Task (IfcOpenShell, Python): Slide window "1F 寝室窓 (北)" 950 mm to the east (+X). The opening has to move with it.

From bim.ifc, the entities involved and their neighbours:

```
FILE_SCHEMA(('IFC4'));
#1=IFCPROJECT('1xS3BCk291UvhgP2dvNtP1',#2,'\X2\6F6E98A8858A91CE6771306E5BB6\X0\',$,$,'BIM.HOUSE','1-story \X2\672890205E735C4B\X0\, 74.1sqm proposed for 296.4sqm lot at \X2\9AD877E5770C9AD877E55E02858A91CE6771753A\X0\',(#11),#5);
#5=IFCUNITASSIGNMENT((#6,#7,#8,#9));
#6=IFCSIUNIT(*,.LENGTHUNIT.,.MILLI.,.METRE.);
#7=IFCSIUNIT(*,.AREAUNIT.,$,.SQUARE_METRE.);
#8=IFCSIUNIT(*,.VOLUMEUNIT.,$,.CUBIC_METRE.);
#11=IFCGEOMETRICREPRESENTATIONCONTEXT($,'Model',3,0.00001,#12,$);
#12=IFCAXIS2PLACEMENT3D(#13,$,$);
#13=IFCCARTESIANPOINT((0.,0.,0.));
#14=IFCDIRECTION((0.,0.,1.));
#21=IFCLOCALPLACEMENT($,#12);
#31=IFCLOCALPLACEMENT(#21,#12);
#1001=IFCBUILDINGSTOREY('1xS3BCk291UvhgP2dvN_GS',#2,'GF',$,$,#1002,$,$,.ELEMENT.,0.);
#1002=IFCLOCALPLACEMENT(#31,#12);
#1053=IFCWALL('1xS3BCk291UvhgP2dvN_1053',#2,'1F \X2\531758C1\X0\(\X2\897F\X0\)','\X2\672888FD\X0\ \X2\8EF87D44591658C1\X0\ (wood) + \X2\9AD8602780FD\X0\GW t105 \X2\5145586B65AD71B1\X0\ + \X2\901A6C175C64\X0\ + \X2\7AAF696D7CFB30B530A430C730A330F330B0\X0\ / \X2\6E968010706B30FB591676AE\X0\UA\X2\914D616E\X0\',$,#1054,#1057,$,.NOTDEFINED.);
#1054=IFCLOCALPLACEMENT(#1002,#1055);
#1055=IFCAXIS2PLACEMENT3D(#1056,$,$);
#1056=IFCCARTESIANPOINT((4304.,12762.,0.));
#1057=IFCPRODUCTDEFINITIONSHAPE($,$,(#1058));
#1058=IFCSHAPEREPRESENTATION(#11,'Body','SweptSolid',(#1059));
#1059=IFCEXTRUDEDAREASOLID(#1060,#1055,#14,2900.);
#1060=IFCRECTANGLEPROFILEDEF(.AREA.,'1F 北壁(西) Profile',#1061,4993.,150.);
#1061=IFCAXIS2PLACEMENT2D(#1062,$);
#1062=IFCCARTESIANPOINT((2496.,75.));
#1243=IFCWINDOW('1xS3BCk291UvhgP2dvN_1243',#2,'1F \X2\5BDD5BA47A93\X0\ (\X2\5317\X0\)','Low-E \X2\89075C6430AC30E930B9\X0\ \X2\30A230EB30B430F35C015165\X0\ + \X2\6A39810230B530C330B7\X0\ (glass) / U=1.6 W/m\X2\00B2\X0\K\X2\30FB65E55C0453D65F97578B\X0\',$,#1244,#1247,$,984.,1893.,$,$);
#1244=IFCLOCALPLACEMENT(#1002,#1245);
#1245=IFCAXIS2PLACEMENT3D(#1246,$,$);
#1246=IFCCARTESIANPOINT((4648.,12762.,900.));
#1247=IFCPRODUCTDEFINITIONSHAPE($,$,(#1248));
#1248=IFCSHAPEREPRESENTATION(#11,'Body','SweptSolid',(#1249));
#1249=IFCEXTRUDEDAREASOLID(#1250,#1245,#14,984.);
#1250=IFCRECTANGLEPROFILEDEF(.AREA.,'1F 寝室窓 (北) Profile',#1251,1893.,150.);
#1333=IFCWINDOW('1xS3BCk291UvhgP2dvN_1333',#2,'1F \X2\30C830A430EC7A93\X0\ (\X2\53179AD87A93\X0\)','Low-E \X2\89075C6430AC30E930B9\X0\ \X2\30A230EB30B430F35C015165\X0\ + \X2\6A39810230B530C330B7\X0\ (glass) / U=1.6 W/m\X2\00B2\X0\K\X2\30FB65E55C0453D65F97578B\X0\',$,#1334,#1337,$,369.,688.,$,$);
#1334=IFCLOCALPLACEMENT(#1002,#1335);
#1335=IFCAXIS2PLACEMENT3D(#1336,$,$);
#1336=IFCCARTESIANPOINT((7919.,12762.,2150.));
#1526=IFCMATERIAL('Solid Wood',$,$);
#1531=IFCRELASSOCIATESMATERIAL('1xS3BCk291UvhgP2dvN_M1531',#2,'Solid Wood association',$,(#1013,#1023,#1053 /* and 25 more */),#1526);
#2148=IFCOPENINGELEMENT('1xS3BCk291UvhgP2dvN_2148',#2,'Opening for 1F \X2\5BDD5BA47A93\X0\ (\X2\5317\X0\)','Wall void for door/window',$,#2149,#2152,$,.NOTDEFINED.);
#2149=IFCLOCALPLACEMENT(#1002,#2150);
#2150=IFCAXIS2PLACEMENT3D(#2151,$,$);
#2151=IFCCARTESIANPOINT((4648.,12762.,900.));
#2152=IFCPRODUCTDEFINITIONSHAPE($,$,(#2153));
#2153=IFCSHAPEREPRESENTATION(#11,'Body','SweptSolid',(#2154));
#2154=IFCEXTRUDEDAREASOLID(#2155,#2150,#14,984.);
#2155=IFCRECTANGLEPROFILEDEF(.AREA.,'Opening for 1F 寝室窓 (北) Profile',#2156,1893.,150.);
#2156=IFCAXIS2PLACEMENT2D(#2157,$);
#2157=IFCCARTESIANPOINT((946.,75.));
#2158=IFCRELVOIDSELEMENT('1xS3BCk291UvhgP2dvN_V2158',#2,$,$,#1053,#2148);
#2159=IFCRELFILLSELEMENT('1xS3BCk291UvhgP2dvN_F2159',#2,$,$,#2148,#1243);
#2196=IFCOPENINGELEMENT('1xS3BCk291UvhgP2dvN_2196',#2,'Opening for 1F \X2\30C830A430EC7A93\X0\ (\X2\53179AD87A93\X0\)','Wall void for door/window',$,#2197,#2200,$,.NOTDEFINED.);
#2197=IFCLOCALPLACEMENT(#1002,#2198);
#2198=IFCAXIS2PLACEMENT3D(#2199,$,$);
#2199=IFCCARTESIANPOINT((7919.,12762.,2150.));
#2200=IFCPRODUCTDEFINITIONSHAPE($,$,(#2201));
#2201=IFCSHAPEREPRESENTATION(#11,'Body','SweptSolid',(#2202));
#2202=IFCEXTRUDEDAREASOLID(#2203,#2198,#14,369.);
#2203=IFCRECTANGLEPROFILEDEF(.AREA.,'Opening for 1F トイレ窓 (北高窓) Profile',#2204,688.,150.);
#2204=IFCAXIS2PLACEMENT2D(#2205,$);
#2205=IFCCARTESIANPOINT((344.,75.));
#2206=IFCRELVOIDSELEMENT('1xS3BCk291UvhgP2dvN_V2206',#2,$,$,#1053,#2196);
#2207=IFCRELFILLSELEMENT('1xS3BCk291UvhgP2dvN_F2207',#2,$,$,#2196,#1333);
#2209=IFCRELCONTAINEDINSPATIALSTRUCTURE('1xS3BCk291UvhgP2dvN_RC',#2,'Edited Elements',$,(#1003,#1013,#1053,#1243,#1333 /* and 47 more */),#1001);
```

```python
import ifcopenshell
import ifcopenshell.api.geometry
import ifcopenshell.util.placement
import ifcopenshell.util.unit

model = ifcopenshell.open("bim.ifc")
unit_scale = ifcopenshell.util.unit.calculate_unit_scale(model)

window = model.by_guid("1xS3BCk291UvhgP2dvN_1243")
opening = window.FillsVoids[0].RelatingOpeningElement
wall = opening.VoidsElements[0].RelatingBuildingElement

wall_matrix = ifcopenshell.util.placement.get_local_placement(wall.ObjectPlacement)
shift = wall_matrix[:3, 0] * 0.95 / unit_scale
before = ifcopenshell.util.placement.get_local_placement(window.ObjectPlacement)[:3, 3].copy()

# The window is not placed relative to its opening, so move both.
for product in (opening, window):
    matrix = ifcopenshell.util.placement.get_local_placement(product.ObjectPlacement)
    matrix[:3, 3] += shift
    ifcopenshell.api.geometry.edit_object_placement(model, product=product, matrix=matrix, is_si=False)

after = ifcopenshell.util.placement.get_local_placement(window.ObjectPlacement)[:3, 3]
print("window moved by", (after - before).round(3) + 0.0)

model.write("bim_updated.ifc")
```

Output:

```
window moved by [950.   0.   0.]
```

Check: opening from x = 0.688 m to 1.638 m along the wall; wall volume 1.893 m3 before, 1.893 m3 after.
